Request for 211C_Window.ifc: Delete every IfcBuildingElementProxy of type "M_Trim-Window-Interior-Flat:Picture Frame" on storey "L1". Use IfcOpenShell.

First a look at what the model holds.

```python
import ifcopenshell
import ifcopenshell.util.element

model = ifcopenshell.open("211C_Window.ifc")
print(model.schema)
storey = next(s for s in model.by_type("IfcBuildingStorey") if s.Name == "L1")
proxies = [e for e in ifcopenshell.util.element.get_decomposition(storey) if e.is_a("IfcBuildingElementProxy")]
seen = {}
for e in proxies:
    element_type = ifcopenshell.util.element.get_type(e)
    name = element_type.Name if element_type not in (None, e) else None
    seen[name] = seen.get(name, 0) + 1
for name, count in sorted(seen.items(), key=str):
    print(count, "x", name)
```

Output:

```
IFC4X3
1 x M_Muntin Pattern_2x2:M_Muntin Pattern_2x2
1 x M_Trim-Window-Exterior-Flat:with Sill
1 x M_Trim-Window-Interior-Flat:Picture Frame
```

```python
import ifcopenshell
import ifcopenshell.api.root
import ifcopenshell.util.element

model = ifcopenshell.open("211C_Window.ifc")

storey = next(s for s in model.by_type("IfcBuildingStorey") if s.Name == "L1")
proxies = [e for e in ifcopenshell.util.element.get_decomposition(storey) if e.is_a("IfcBuildingElementProxy")]
targets = [e for e in proxies if (t := ifcopenshell.util.element.get_type(e)) not in (None, e) and t.Name == "M_Trim-Window-Interior-Flat:Picture Frame"]

for e in targets:
    ifcopenshell.api.root.remove_product(model, product=e)
print(len(targets), "removed")

model.write("211C_Window_updated.ifc")
```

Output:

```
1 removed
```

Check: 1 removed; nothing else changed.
